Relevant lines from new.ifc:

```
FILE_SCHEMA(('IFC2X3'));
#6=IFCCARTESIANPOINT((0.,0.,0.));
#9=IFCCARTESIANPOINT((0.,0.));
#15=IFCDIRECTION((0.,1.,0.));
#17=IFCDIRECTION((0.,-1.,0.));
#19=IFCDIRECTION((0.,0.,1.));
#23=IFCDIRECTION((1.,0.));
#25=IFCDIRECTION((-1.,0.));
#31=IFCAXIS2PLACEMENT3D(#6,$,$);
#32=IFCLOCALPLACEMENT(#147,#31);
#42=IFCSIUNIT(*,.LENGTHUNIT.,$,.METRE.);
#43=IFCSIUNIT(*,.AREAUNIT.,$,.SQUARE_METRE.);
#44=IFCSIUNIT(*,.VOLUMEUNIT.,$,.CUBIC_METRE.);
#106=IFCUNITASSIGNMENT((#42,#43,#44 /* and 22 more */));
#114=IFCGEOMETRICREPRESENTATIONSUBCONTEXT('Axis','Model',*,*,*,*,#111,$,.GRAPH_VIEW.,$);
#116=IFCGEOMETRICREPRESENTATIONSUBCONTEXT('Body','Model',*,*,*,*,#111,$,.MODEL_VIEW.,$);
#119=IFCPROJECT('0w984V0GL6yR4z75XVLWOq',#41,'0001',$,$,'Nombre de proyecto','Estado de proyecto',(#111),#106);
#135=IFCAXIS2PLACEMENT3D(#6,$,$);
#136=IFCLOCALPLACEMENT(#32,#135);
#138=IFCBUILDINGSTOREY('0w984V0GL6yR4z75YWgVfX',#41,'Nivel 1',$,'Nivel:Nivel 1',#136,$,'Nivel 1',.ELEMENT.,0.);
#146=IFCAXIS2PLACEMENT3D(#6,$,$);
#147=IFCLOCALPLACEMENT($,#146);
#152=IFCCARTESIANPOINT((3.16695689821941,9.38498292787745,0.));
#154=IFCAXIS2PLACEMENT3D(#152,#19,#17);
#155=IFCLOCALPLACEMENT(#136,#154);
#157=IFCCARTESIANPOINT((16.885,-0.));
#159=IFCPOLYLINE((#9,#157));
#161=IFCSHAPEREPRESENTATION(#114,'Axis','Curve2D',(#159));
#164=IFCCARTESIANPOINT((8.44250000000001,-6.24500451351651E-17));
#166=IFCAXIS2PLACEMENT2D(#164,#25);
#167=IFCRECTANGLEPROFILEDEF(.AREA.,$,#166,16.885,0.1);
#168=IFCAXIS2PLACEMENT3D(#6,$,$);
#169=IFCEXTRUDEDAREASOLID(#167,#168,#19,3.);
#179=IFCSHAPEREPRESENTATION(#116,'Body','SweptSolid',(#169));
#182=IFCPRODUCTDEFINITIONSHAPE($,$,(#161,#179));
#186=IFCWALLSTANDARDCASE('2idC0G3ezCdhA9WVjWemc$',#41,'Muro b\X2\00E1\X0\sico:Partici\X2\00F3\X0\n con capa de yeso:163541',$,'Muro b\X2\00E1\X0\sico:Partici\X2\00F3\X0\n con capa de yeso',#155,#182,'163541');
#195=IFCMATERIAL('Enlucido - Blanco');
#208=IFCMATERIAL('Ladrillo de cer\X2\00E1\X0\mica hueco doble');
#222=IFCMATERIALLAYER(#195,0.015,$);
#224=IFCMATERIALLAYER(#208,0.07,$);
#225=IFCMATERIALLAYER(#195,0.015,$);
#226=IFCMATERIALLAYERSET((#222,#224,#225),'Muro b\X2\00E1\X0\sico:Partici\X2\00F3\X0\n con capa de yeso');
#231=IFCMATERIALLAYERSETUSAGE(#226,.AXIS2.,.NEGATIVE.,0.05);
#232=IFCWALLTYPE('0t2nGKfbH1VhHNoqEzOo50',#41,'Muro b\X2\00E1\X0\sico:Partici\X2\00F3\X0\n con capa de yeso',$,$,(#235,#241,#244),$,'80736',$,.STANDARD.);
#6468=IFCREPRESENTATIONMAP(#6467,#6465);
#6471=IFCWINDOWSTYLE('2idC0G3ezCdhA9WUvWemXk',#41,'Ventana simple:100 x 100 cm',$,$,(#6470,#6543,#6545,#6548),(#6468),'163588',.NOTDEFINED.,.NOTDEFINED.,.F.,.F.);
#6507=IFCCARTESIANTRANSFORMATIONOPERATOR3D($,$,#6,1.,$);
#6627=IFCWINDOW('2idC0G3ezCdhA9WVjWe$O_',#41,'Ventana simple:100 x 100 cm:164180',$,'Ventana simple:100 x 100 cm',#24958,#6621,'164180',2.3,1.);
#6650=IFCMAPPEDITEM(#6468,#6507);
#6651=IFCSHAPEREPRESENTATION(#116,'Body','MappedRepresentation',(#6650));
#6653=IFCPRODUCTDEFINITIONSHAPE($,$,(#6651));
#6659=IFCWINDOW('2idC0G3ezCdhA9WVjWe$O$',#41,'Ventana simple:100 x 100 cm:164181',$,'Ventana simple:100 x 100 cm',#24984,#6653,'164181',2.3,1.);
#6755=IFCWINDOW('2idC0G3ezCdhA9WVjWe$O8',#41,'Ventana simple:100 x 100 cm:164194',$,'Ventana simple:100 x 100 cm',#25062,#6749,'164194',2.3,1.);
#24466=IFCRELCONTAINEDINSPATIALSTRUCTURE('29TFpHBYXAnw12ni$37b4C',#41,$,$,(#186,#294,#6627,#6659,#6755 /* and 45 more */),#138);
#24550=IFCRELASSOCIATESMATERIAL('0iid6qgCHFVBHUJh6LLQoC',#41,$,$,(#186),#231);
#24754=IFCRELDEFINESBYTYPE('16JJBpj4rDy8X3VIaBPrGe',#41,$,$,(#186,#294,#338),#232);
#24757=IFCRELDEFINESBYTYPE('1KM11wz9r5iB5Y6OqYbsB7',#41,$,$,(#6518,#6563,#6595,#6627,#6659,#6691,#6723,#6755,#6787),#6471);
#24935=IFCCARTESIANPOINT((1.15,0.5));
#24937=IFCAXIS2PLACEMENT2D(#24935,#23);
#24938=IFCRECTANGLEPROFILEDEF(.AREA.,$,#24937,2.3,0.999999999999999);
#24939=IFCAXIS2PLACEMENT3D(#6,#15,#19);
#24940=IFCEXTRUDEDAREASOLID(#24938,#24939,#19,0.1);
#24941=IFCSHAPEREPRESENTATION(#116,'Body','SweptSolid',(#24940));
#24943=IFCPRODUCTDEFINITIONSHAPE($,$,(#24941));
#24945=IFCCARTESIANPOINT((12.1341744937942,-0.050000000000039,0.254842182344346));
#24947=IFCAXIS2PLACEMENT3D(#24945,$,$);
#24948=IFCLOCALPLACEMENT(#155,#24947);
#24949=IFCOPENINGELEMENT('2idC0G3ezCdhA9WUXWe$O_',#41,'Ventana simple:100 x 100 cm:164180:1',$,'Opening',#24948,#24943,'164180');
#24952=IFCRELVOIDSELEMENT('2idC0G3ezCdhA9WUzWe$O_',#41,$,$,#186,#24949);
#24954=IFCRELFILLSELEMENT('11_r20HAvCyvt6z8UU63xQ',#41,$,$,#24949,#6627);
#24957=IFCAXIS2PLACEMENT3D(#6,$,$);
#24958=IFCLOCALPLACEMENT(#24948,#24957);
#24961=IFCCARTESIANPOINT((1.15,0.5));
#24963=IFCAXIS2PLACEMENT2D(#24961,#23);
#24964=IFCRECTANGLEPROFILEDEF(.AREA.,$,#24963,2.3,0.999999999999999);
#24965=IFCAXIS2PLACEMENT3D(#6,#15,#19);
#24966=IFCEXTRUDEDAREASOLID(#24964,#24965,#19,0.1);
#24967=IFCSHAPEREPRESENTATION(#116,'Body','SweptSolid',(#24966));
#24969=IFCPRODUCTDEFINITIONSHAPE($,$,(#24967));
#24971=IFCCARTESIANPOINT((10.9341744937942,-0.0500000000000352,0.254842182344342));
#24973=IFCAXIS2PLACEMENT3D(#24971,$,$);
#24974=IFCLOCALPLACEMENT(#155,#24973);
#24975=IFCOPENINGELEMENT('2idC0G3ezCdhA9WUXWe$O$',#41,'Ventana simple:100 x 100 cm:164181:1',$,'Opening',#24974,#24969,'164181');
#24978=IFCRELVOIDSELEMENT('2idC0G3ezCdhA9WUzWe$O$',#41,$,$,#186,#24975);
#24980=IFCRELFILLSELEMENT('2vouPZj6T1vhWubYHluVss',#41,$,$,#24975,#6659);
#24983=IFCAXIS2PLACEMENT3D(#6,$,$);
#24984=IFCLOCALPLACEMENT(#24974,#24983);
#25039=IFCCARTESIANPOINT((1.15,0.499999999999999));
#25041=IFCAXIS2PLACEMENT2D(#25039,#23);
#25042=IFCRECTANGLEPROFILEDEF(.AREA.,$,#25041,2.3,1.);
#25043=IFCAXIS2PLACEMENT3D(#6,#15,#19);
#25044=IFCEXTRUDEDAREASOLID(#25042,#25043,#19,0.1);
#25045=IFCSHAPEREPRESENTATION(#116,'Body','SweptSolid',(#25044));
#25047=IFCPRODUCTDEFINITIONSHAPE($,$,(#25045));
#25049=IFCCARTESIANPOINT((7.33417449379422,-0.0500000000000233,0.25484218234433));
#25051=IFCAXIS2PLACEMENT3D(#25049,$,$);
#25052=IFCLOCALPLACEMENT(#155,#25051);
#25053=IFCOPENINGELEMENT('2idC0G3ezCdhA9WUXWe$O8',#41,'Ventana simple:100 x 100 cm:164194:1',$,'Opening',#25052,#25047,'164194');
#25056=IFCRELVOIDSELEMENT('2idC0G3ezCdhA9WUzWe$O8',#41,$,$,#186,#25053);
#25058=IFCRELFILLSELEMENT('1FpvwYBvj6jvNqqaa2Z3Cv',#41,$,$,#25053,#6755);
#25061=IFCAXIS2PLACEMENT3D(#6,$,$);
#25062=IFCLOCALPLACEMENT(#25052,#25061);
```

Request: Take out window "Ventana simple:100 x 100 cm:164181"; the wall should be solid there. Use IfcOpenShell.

```python
import ifcopenshell
import ifcopenshell.api.feature
import ifcopenshell.api.root
import ifcopenshell.geom
import ifcopenshell.util.shape

model = ifcopenshell.open("new.ifc")
settings = ifcopenshell.geom.settings()


def volume(element):
    """Net volume in cubic metres, openings subtracted."""
    shape = ifcopenshell.geom.create_shape(settings, element)
    return ifcopenshell.util.shape.get_volume(shape.geometry)


window = model.by_guid("2idC0G3ezCdhA9WVjWe$O$")
opening = window.FillsVoids[0].RelatingOpeningElement
wall = opening.VoidsElements[0].RelatingBuildingElement
before = volume(wall)

ifcopenshell.api.root.remove_product(model, product=window)
ifcopenshell.api.feature.remove_feature(model, feature=opening)

after = volume(wall)

print(f"wall volume {before:.3f} -> {after:.3f} m3")

model.write("new_edited.ifc")
```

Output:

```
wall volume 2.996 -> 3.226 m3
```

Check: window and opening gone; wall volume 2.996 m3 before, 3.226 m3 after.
